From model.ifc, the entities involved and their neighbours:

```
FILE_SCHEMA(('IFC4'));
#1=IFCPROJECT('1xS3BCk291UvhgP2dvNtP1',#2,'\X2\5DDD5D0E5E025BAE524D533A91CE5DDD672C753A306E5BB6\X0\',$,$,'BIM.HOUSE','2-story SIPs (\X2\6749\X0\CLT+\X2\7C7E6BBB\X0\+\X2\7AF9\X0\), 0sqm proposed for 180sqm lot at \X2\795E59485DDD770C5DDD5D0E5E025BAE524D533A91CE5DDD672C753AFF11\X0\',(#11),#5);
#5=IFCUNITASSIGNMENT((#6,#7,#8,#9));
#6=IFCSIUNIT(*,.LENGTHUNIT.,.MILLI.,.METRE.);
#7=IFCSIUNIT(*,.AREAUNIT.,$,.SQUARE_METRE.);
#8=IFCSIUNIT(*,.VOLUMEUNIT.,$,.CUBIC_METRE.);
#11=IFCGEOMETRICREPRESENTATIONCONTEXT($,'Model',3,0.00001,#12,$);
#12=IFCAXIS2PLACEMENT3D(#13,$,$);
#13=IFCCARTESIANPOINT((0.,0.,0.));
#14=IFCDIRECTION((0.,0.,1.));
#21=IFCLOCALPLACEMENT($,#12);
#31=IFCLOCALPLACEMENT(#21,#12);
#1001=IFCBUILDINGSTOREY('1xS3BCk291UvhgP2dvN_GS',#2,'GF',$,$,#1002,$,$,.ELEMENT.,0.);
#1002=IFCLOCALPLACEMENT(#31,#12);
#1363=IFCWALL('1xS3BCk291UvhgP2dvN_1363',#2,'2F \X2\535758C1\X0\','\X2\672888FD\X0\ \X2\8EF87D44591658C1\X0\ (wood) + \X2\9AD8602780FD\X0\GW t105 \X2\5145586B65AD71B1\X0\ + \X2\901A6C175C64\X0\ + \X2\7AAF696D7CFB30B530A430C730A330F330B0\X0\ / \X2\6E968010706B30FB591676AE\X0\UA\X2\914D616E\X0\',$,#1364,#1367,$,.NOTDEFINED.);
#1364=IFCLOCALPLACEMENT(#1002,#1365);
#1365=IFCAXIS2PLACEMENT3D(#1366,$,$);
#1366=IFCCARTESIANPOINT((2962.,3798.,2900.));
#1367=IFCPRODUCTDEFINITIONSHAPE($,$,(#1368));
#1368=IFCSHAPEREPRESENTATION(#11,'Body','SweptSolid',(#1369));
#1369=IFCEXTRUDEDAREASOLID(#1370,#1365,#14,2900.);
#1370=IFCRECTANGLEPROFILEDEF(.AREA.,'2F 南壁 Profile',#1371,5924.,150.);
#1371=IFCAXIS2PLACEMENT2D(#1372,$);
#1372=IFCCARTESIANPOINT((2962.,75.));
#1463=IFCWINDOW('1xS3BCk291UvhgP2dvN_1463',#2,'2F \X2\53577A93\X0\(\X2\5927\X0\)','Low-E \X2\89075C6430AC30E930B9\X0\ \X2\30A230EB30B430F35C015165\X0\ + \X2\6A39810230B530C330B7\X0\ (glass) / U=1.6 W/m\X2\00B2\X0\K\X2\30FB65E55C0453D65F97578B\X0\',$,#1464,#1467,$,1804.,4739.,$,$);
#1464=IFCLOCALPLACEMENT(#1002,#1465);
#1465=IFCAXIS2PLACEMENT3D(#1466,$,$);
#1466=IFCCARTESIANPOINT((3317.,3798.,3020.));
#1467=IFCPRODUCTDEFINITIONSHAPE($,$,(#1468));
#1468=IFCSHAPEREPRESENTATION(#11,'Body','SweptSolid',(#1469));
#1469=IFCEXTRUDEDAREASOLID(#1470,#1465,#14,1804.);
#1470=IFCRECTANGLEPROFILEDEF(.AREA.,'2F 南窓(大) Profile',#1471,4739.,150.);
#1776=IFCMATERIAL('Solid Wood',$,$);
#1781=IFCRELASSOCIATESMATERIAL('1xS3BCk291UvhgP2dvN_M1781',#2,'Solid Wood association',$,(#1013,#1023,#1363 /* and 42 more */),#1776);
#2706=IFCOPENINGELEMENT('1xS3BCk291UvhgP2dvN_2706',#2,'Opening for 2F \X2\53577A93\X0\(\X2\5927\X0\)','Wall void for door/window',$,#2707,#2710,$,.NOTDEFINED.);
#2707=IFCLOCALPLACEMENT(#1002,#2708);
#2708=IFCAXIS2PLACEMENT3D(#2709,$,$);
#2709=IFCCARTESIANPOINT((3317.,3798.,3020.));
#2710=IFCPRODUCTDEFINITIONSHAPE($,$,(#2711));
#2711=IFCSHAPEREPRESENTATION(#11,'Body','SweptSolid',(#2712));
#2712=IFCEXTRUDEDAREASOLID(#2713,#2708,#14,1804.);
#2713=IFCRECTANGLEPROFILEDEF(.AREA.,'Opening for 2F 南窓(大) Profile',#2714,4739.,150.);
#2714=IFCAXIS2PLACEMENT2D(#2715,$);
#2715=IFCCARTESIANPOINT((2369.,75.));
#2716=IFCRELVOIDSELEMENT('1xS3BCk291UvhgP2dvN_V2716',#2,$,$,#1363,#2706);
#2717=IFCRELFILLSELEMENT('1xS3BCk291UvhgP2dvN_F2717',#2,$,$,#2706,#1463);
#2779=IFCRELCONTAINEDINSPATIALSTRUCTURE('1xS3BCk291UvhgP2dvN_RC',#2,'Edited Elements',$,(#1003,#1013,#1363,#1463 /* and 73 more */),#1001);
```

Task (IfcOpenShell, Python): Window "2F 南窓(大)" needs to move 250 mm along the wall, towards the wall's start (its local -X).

```python
import ifcopenshell
import ifcopenshell.api.geometry
import ifcopenshell.util.placement
import ifcopenshell.util.unit

model = ifcopenshell.open("model.ifc")
unit_scale = ifcopenshell.util.unit.calculate_unit_scale(model)

window = model.by_guid("1xS3BCk291UvhgP2dvN_1463")
opening = window.FillsVoids[0].RelatingOpeningElement
wall = opening.VoidsElements[0].RelatingBuildingElement

wall_matrix = ifcopenshell.util.placement.get_local_placement(wall.ObjectPlacement)
shift = wall_matrix[:3, 0] * -0.25 / unit_scale
before = ifcopenshell.util.placement.get_local_placement(window.ObjectPlacement)[:3, 3].copy()

# The window is not placed relative to its opening, so move both.
for product in (opening, window):
    matrix = ifcopenshell.util.placement.get_local_placement(product.ObjectPlacement)
    matrix[:3, 3] += shift
    ifcopenshell.api.geometry.edit_object_placement(model, product=product, matrix=matrix, is_si=False)

after = ifcopenshell.util.placement.get_local_placement(window.ObjectPlacement)[:3, 3]
print("window moved by", (after - before).round(3) + 0.0)

model.write("model-out.ifc")
```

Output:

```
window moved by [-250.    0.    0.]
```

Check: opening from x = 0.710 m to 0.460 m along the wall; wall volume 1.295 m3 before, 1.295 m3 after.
